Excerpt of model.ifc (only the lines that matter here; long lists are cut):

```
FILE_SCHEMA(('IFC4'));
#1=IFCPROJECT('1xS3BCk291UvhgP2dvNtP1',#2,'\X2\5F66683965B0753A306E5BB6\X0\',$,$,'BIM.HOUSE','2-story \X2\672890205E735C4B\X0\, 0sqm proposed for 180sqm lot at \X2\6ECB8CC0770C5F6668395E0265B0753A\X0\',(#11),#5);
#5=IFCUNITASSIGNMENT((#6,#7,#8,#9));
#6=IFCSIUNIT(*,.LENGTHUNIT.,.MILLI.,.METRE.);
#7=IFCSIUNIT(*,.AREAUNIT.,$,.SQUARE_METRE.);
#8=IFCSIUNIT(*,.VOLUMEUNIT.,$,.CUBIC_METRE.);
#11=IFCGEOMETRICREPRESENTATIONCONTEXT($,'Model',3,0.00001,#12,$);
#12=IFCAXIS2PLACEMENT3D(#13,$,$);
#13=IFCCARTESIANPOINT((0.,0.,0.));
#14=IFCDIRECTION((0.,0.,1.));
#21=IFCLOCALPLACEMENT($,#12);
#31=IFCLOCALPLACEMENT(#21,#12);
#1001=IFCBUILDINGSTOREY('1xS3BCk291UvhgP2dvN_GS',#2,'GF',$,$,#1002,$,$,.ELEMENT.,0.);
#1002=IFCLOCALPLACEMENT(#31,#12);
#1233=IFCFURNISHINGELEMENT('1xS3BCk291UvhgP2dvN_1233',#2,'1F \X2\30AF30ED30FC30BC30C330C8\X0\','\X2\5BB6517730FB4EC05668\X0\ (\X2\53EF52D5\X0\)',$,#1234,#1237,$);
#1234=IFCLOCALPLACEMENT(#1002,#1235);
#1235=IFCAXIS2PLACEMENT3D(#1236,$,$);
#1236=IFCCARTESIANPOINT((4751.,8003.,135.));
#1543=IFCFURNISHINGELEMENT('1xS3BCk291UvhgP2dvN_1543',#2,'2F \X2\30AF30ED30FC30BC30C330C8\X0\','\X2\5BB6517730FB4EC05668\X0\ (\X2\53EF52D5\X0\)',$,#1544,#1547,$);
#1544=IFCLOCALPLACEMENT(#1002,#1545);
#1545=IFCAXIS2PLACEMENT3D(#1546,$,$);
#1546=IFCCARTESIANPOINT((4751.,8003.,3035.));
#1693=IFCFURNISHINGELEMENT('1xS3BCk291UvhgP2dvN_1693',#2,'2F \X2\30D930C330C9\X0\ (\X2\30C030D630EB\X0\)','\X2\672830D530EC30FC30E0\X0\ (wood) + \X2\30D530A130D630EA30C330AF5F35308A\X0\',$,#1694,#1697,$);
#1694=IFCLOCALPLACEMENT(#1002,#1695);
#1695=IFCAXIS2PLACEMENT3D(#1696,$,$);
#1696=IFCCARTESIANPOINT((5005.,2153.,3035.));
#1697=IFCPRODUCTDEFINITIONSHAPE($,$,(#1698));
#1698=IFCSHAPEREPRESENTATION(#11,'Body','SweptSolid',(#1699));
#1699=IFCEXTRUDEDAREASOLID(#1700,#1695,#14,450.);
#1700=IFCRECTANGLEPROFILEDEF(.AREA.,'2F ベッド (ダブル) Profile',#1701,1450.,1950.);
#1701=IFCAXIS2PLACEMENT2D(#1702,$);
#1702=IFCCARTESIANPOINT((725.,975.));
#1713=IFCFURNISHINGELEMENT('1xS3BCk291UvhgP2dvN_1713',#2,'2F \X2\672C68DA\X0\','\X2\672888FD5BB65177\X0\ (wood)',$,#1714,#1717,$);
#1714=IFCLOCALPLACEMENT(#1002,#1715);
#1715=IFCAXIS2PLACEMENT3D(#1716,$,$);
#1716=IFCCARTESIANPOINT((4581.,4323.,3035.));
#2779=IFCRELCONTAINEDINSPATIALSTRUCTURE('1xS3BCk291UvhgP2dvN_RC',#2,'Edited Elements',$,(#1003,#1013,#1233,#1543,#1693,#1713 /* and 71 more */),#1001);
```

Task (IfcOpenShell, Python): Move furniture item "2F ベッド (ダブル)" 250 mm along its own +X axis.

```python
import ifcopenshell
import ifcopenshell.api.geometry
import ifcopenshell.util.placement
import ifcopenshell.util.unit

model = ifcopenshell.open("model.ifc")
unit_scale = ifcopenshell.util.unit.calculate_unit_scale(model)

item = model.by_id(1693)
matrix = ifcopenshell.util.placement.get_local_placement(item.ObjectPlacement)
matrix[:3, 3] += matrix[:3, 0] * 0.25 / unit_scale
ifcopenshell.api.geometry.edit_object_placement(model, product=item, matrix=matrix, is_si=False)

print(ifcopenshell.util.placement.get_local_placement(item.ObjectPlacement).round(3) + 0.0)

model.write("model_edited.ifc")
```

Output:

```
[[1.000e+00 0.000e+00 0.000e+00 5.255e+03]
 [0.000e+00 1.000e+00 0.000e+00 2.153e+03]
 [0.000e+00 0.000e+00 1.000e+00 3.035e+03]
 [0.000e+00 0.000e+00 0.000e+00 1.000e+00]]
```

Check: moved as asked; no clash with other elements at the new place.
